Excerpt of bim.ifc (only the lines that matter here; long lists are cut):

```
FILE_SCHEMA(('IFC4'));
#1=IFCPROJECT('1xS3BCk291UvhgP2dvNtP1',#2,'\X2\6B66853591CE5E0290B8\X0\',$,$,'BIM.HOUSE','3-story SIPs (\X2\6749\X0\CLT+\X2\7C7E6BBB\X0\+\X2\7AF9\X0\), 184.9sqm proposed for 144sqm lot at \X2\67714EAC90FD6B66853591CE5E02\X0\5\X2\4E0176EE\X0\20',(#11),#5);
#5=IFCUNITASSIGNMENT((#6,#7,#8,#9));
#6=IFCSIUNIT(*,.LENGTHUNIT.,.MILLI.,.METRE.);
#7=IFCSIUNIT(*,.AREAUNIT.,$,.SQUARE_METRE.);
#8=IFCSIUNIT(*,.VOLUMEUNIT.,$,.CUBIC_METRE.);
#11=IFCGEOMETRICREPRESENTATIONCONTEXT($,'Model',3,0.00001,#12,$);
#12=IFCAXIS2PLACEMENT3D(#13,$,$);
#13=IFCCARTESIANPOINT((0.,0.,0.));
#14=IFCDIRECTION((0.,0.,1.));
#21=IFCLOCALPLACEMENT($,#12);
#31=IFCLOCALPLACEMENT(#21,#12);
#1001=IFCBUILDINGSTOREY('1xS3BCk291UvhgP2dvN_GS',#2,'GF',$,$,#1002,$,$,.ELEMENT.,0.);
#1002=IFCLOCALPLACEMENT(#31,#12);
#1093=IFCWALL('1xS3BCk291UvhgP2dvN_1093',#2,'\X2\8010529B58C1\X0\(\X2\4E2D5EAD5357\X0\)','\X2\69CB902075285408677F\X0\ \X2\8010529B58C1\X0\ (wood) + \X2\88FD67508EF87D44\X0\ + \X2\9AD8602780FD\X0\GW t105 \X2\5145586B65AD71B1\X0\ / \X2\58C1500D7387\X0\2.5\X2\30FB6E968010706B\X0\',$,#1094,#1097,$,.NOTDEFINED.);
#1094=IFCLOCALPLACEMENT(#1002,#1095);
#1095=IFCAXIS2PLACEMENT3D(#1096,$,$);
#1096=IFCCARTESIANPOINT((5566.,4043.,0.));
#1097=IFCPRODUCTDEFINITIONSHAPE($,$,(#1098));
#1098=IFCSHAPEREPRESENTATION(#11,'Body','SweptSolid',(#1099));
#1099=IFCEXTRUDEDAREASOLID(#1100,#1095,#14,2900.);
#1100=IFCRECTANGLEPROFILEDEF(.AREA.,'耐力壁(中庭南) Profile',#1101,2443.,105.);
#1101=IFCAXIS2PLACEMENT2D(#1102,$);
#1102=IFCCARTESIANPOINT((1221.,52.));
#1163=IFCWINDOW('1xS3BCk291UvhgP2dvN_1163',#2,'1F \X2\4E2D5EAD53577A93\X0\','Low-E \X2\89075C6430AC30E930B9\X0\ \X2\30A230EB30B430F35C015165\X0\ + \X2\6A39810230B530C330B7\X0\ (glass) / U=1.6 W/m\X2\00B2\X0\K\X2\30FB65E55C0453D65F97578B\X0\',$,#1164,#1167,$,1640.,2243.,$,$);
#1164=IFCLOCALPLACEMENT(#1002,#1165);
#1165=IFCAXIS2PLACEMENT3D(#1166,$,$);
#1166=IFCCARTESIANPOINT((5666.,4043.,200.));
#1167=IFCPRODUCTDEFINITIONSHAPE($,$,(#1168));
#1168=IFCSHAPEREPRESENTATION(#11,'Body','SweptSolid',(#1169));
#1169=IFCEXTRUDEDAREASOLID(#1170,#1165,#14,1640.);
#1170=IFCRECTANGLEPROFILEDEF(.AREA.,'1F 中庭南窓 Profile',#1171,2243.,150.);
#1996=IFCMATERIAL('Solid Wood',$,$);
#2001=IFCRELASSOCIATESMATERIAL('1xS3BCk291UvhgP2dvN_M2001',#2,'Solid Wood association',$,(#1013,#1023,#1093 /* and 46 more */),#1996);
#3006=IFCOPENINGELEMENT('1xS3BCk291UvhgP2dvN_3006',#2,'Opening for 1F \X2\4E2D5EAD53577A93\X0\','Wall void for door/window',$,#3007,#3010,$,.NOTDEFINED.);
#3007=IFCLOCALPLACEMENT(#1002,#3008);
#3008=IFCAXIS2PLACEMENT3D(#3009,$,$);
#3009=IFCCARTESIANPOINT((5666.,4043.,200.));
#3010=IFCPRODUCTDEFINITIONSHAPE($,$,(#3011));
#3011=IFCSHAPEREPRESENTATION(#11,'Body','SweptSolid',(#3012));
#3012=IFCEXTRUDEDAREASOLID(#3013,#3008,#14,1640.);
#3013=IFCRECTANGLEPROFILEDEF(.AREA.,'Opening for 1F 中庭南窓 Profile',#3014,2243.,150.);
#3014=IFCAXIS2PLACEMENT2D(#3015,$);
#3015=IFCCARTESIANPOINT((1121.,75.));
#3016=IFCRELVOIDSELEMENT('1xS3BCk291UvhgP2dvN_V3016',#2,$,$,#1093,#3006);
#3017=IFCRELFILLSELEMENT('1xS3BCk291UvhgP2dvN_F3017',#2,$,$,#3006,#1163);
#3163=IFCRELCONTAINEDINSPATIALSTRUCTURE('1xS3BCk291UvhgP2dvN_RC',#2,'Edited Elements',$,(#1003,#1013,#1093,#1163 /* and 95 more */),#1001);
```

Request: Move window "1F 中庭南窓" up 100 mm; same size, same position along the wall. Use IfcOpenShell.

```python
import numpy as np
import ifcopenshell
import ifcopenshell.api.geometry
import ifcopenshell.util.placement
import ifcopenshell.util.unit

model = ifcopenshell.open("bim.ifc")
unit_scale = ifcopenshell.util.unit.calculate_unit_scale(model)

window = model.by_id(1163)
opening = window.FillsVoids[0].RelatingOpeningElement
dz = 100.0

shift = np.array([0.0, 0.0, dz])
# The window is not placed relative to its opening, so move both.
for product in (opening, window):
    matrix = ifcopenshell.util.placement.get_local_placement(product.ObjectPlacement)
    matrix[:3, 3] += shift
    ifcopenshell.api.geometry.edit_object_placement(model, product=product, matrix=matrix, is_si=False)

print(f"moved by {dz * unit_scale:+.3f} m")

model.write("bim_rev.ifc")
```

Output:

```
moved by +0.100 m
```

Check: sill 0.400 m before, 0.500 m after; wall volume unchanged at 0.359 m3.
